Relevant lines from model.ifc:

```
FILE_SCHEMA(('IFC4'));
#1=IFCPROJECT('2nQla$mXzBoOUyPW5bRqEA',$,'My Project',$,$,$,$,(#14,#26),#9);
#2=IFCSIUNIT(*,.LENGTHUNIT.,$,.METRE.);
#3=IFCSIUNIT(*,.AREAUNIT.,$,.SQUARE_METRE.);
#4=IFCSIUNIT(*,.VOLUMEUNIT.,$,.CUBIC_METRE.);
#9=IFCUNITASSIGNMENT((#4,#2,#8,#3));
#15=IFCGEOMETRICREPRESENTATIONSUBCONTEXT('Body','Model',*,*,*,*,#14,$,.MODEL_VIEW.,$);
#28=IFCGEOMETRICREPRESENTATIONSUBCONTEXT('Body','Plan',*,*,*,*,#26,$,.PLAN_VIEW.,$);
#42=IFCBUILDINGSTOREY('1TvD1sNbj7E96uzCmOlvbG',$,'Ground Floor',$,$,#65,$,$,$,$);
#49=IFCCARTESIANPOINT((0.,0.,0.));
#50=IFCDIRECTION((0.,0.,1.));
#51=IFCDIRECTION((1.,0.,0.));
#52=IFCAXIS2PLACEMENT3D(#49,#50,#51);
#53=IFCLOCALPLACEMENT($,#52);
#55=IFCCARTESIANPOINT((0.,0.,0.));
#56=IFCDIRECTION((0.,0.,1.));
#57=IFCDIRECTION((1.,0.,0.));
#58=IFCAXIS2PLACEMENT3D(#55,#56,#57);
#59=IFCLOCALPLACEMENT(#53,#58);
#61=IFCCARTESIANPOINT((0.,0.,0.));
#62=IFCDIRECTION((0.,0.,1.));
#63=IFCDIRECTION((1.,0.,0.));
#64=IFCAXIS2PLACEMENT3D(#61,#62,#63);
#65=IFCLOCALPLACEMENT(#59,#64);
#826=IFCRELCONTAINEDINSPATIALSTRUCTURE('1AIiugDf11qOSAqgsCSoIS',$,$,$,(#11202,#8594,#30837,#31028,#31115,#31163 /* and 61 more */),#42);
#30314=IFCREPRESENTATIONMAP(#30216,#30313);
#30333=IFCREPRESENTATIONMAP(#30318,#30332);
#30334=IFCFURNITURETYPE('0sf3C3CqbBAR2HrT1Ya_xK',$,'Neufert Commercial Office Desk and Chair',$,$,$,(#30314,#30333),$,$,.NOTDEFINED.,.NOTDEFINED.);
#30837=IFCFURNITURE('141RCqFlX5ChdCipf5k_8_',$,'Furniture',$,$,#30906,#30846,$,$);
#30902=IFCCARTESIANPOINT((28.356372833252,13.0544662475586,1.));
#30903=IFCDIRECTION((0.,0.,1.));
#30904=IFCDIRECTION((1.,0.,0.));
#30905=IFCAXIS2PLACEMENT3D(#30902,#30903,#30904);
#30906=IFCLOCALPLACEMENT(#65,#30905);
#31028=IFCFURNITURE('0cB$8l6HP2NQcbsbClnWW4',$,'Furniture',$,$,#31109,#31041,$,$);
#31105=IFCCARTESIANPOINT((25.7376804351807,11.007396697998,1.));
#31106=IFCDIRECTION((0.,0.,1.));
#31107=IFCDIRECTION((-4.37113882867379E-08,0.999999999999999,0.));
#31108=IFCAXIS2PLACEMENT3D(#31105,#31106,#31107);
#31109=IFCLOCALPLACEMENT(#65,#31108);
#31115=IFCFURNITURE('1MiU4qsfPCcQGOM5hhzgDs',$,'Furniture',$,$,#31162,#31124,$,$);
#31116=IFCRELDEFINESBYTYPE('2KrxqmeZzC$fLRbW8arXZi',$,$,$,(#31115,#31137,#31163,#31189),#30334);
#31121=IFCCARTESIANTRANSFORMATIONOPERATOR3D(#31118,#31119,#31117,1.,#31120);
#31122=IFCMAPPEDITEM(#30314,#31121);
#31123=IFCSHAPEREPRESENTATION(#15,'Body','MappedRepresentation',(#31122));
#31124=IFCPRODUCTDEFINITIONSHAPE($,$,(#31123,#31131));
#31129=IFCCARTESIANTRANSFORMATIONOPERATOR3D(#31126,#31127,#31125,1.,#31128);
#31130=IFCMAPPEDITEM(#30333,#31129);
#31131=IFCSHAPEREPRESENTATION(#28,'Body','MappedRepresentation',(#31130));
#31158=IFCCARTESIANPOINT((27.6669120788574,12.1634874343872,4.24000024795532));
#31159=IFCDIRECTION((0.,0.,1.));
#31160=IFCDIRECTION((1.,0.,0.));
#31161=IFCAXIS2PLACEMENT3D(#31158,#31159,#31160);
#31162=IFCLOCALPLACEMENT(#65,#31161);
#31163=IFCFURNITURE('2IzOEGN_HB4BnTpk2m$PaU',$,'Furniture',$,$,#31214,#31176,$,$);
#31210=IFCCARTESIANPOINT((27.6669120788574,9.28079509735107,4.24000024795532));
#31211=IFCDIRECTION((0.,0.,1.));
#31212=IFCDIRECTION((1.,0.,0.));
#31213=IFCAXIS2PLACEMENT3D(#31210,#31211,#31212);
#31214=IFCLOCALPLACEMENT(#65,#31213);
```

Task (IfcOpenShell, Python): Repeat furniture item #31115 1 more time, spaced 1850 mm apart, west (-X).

```python
import numpy as np
import ifcopenshell
import ifcopenshell.api.geometry
import ifcopenshell.api.root
import ifcopenshell.util.element
import ifcopenshell.util.placement
import ifcopenshell.util.unit

model = ifcopenshell.open("model.ifc")
unit_scale = ifcopenshell.util.unit.calculate_unit_scale(model)

source = model.by_guid("1MiU4qsfPCcQGOM5hhzgDs")
base = ifcopenshell.util.placement.get_local_placement(source.ObjectPlacement)
step = np.array([-1.0, 0.0, 0.0]) * 1.85 / unit_scale

for i in range(1, 2):
    copy = ifcopenshell.api.root.copy_class(model, product=source)
    copy.Representation = ifcopenshell.util.element.copy_deep(
        model, source.Representation, exclude=["IfcGeometricRepresentationContext", "IfcRepresentationMap"]
    )
    matrix = base.copy()
    matrix[:3, 3] += i * step
    print("added at", matrix[:3, 3].round(3) + 0.0)
    ifcopenshell.api.geometry.edit_object_placement(model, product=copy, matrix=matrix, is_si=False)

model.write("model_rev.ifc")
```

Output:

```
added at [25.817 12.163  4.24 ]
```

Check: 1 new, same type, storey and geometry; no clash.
